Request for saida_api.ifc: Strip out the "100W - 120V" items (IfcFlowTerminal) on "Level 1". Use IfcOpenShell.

First a look at what the model holds.

```python
import ifcopenshell
import ifcopenshell.util.element

model = ifcopenshell.open("saida_api.ifc")
print(model.schema)
storey = next(s for s in model.by_type("IfcBuildingStorey") if s.Name == "Level 1")
terminals = [e for e in ifcopenshell.util.element.get_decomposition(storey) if e.is_a("IfcFlowTerminal")]
seen = {}
for e in terminals:
    element_type = ifcopenshell.util.element.get_type(e)
    name = element_type.Name if element_type not in (None, e) else None
    seen[name] = seen.get(name, 0) + 1
for name, count in sorted(seen.items(), key=str):
    print(count, "x", name)
```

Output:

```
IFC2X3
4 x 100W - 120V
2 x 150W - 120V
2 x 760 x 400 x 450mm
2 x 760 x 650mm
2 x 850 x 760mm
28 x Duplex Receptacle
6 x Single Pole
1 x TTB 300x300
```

```python
import ifcopenshell
import ifcopenshell.api.root
import ifcopenshell.util.element

model = ifcopenshell.open("saida_api.ifc")

storey = next(s for s in model.by_type("IfcBuildingStorey") if s.Name == "Level 1")
terminals = [e for e in ifcopenshell.util.element.get_decomposition(storey) if e.is_a("IfcFlowTerminal")]
targets = [e for e in terminals if (t := ifcopenshell.util.element.get_type(e)) not in (None, e) and t.Name == "100W - 120V"]

for e in targets:
    ifcopenshell.api.root.remove_product(model, product=e)
print(len(targets), "removed")

model.write("saida_api_edited.ifc")
```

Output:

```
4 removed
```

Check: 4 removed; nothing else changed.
